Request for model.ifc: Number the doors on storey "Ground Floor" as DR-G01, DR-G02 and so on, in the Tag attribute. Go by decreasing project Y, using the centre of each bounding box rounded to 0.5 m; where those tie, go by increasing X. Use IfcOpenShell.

First a look at what the model holds.

```python
import ifcopenshell
import ifcopenshell.util.element
import ifcopenshell.util.placement

model = ifcopenshell.open("model.ifc")
print(model.schema)
storey = next(s for s in model.by_type("IfcBuildingStorey") if s.Name == "Ground Floor")
doors = [e for e in ifcopenshell.util.element.get_decomposition(storey) if e.is_a("IfcDoor")]
for e in sorted(doors, key=lambda e: e.id()):
    origin = ifcopenshell.util.placement.get_local_placement(e.ObjectPlacement)[:3, 3]
    print(e.id(), e.Tag, e.Name, origin.round(2) + 0.0, sep=" | ")
```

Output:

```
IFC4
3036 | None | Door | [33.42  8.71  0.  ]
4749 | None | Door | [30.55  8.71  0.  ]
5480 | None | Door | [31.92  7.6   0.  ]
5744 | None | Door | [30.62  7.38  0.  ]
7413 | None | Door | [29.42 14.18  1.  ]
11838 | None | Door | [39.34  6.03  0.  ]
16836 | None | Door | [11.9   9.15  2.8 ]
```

```python
import ifcopenshell
import ifcopenshell.geom
import ifcopenshell.util.element
import ifcopenshell.util.shape

model = ifcopenshell.open("model.ifc")
settings = ifcopenshell.geom.settings()
settings.set("use-world-coords", True)


def centre(element):
    shape = ifcopenshell.geom.create_shape(settings, element)
    return ifcopenshell.util.shape.get_bbox_centroid(shape.geometry)


storey = next(s for s in model.by_type("IfcBuildingStorey") if s.Name == "Ground Floor")
doors = [e for e in ifcopenshell.util.element.get_decomposition(storey) if e.is_a("IfcDoor")]

# Insertion points can sit at a corner or the storey origin, so sort by the geometry (in metres).
centres = {e: centre(e) for e in doors}
doors.sort(key=lambda e: (-round(centres[e][1] / 0.5), centres[e][0]))

for i, e in enumerate(doors, start=1):
    number = f"DR-G{i:02d}"
    e.Tag = number
    print(e.id(), number)

model.write("model_v2.ifc")
```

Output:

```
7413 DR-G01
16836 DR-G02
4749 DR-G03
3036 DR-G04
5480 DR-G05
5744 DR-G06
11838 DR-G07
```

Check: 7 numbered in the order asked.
